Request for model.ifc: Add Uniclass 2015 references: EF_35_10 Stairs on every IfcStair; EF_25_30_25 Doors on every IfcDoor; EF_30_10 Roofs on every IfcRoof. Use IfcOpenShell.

First a look at what the model holds.

```python
import ifcopenshell

model = ifcopenshell.open("model.ifc")
print(model.schema)
print("classifications:", [c.Name for c in model.by_type("IfcClassification")])
for ifc_class in ("IfcDoor", "IfcRoof", "IfcStair", "IfcWall", "IfcWindow"):
    print(ifc_class, len(model.by_type(ifc_class)))
```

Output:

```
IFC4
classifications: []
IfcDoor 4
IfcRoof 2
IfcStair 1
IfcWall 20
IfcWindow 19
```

```python
import ifcopenshell
import ifcopenshell.api.classification

model = ifcopenshell.open("model.ifc")

system = ifcopenshell.api.classification.add_classification(model, classification="Uniclass 2015")

codes = {
    "IfcStair": ("EF_35_10", "Stairs"),
    "IfcDoor": ("EF_25_30_25", "Doors"),
    "IfcRoof": ("EF_30_10", "Roofs"),
}
for ifc_class, (code, name) in codes.items():
    products = model.by_type(ifc_class)
    ifcopenshell.api.classification.add_reference(
        model, products=products, classification=system, identification=code, name=name
    )
    print(code, len(products))

model.write("model_rev.ifc")
```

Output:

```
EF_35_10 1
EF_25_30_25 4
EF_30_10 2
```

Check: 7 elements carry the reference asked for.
